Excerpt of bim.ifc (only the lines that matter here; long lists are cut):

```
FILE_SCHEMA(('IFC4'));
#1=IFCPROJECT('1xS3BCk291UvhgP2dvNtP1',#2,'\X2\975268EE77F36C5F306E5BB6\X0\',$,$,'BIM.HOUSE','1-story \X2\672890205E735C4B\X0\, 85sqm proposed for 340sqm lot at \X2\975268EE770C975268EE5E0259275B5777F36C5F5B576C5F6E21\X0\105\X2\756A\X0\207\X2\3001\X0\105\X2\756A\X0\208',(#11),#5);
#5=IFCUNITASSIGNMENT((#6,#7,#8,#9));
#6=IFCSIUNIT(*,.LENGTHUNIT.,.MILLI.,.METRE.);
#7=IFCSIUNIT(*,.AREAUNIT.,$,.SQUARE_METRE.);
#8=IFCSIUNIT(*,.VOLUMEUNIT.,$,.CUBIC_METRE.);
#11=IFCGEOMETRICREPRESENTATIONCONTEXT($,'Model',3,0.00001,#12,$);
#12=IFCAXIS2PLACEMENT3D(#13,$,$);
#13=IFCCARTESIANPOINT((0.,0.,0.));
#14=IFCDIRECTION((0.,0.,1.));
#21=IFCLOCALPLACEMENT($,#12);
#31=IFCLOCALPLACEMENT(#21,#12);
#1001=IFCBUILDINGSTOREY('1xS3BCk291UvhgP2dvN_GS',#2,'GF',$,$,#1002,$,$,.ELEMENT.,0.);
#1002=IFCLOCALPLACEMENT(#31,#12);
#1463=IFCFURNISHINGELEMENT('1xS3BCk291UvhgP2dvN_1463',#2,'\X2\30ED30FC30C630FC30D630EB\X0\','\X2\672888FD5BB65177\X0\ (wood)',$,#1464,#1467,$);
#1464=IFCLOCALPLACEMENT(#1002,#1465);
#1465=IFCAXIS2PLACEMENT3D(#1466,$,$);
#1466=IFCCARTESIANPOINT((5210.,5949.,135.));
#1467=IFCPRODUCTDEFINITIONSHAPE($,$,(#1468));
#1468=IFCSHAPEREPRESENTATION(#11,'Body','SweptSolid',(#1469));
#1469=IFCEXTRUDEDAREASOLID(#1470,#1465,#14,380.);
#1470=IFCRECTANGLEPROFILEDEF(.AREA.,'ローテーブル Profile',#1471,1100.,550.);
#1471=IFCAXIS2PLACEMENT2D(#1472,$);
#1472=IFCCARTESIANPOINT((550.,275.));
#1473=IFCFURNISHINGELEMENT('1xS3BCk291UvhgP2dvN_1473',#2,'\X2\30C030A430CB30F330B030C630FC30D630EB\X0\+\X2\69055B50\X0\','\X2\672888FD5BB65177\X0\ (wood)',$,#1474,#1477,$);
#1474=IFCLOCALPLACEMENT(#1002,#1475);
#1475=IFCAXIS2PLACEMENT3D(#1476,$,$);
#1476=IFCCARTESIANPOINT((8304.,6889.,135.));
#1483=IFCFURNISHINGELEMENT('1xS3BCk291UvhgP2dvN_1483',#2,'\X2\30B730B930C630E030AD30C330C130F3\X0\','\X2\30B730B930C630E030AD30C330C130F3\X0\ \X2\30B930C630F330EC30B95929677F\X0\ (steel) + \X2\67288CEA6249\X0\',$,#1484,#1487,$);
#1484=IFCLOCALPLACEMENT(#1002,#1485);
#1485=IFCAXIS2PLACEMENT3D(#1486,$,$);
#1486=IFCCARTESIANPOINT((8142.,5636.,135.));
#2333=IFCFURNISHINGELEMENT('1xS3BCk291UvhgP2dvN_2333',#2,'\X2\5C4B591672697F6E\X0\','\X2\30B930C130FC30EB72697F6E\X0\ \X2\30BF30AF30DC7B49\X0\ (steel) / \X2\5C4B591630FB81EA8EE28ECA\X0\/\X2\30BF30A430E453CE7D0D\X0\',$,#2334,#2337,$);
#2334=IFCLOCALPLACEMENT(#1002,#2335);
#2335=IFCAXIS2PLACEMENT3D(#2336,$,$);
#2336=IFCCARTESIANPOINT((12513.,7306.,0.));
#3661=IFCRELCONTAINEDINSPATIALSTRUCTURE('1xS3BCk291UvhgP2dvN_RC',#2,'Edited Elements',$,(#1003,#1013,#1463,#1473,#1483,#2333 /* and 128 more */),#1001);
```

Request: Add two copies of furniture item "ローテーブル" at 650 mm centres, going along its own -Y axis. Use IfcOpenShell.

```python
import ifcopenshell
import ifcopenshell.api.geometry
import ifcopenshell.api.root
import ifcopenshell.util.element
import ifcopenshell.util.placement
import ifcopenshell.util.unit

model = ifcopenshell.open("bim.ifc")
unit_scale = ifcopenshell.util.unit.calculate_unit_scale(model)


def reuse_history(source, copy):
    """copy_class also copies each property set's owner history, people and application; keep the originals."""
    for rel in copy.IsDefinedBy:
        if rel.is_a("IfcRelDefinesByProperties") and (history := rel.RelatingPropertyDefinition.OwnerHistory):
            rel.RelatingPropertyDefinition.OwnerHistory = source.OwnerHistory
            ifcopenshell.util.element.remove_deep2(model, history)


source = model.by_guid("1xS3BCk291UvhgP2dvN_1463")
base = ifcopenshell.util.placement.get_local_placement(source.ObjectPlacement)
step = -base[:3, 1] * 0.65 / unit_scale

for i in range(1, 3):
    copy = ifcopenshell.api.root.copy_class(model, product=source)
    copy.Representation = ifcopenshell.util.element.copy_deep(
        model, source.Representation, exclude=["IfcGeometricRepresentationContext", "IfcRepresentationMap"]
    )
    reuse_history(source, copy)
    matrix = base.copy()
    matrix[:3, 3] += i * step
    print("added at", matrix[:3, 3].round(3) + 0.0)
    ifcopenshell.api.geometry.edit_object_placement(model, product=copy, matrix=matrix, is_si=False)

model.write("bim-out.ifc")
```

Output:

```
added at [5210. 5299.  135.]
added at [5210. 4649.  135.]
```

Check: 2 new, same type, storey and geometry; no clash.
